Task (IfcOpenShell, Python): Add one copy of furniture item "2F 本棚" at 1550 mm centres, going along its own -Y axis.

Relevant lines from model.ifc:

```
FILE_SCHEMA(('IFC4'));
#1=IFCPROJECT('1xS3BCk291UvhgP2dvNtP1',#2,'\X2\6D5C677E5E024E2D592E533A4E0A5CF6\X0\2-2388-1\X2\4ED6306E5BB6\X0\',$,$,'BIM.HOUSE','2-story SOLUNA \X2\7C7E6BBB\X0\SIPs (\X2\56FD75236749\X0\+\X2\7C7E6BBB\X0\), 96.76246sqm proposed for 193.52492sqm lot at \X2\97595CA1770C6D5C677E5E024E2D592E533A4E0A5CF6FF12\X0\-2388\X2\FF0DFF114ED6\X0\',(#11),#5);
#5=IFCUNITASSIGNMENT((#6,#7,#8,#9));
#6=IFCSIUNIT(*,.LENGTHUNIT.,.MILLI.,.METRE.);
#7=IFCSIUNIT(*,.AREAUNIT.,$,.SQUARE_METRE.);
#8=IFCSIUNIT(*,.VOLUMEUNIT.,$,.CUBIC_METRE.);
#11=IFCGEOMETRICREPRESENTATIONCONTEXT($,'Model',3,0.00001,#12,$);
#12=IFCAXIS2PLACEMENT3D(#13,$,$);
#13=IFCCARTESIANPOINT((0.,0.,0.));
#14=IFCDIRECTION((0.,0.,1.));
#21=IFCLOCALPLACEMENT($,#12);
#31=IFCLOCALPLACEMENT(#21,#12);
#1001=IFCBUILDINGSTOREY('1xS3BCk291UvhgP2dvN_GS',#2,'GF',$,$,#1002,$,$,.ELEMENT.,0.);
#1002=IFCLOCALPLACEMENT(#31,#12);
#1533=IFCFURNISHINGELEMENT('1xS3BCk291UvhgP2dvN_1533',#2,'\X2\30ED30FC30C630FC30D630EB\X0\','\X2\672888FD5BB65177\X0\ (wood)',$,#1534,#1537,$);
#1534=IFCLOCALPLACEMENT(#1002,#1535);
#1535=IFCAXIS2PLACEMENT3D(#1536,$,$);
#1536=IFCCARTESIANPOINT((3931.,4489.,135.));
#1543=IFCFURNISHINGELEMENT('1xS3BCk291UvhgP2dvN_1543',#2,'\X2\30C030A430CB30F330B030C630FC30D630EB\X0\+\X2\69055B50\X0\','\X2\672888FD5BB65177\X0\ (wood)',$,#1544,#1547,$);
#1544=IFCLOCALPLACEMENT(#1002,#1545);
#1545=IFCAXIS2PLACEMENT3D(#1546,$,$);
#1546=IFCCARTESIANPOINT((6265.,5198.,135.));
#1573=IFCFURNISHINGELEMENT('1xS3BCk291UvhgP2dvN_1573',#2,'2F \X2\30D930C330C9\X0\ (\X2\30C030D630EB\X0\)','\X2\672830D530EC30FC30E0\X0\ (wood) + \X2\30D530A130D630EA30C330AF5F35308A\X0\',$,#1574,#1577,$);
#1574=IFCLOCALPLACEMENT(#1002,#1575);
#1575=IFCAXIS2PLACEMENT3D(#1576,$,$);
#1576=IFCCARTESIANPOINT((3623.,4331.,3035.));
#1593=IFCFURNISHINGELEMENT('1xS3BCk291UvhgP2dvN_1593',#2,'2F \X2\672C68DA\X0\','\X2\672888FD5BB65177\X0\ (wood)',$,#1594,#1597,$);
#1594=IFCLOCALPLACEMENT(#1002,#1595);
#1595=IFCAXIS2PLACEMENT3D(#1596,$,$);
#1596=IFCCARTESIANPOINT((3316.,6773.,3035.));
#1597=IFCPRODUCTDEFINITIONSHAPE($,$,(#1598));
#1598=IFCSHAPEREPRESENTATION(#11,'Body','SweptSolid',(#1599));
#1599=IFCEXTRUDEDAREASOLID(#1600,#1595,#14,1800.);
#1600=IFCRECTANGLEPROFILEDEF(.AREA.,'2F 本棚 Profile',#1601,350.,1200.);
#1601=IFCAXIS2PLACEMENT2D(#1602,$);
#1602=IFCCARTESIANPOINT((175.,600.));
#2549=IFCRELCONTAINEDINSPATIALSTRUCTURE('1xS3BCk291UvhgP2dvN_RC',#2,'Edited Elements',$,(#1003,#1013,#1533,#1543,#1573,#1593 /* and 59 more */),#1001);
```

```python
import ifcopenshell
import ifcopenshell.api.geometry
import ifcopenshell.api.root
import ifcopenshell.util.element
import ifcopenshell.util.placement

model = ifcopenshell.open("model.ifc")


def reuse_history(source, copy):
    """copy_class also copies each property set's owner history, people and application; keep the originals."""
    for rel in copy.IsDefinedBy:
        if rel.is_a("IfcRelDefinesByProperties") and (history := rel.RelatingPropertyDefinition.OwnerHistory):
            rel.RelatingPropertyDefinition.OwnerHistory = source.OwnerHistory
            ifcopenshell.util.element.remove_deep2(model, history)


source = model.by_guid("1xS3BCk291UvhgP2dvN_1593")
base = ifcopenshell.util.placement.get_local_placement(source.ObjectPlacement)
step = -base[:3, 1] * 1550.0

for i in range(1, 2):
    copy = ifcopenshell.api.root.copy_class(model, product=source)
    copy.Representation = ifcopenshell.util.element.copy_deep(
        model, source.Representation, exclude=["IfcGeometricRepresentationContext", "IfcRepresentationMap"]
    )
    reuse_history(source, copy)
    matrix = base.copy()
    matrix[:3, 3] += i * step
    print("added at", matrix[:3, 3].round(3) + 0.0)
    ifcopenshell.api.geometry.edit_object_placement(model, product=copy, matrix=matrix, is_si=False)

model.write("model-out.ifc")
```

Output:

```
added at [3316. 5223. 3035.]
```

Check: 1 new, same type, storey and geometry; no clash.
